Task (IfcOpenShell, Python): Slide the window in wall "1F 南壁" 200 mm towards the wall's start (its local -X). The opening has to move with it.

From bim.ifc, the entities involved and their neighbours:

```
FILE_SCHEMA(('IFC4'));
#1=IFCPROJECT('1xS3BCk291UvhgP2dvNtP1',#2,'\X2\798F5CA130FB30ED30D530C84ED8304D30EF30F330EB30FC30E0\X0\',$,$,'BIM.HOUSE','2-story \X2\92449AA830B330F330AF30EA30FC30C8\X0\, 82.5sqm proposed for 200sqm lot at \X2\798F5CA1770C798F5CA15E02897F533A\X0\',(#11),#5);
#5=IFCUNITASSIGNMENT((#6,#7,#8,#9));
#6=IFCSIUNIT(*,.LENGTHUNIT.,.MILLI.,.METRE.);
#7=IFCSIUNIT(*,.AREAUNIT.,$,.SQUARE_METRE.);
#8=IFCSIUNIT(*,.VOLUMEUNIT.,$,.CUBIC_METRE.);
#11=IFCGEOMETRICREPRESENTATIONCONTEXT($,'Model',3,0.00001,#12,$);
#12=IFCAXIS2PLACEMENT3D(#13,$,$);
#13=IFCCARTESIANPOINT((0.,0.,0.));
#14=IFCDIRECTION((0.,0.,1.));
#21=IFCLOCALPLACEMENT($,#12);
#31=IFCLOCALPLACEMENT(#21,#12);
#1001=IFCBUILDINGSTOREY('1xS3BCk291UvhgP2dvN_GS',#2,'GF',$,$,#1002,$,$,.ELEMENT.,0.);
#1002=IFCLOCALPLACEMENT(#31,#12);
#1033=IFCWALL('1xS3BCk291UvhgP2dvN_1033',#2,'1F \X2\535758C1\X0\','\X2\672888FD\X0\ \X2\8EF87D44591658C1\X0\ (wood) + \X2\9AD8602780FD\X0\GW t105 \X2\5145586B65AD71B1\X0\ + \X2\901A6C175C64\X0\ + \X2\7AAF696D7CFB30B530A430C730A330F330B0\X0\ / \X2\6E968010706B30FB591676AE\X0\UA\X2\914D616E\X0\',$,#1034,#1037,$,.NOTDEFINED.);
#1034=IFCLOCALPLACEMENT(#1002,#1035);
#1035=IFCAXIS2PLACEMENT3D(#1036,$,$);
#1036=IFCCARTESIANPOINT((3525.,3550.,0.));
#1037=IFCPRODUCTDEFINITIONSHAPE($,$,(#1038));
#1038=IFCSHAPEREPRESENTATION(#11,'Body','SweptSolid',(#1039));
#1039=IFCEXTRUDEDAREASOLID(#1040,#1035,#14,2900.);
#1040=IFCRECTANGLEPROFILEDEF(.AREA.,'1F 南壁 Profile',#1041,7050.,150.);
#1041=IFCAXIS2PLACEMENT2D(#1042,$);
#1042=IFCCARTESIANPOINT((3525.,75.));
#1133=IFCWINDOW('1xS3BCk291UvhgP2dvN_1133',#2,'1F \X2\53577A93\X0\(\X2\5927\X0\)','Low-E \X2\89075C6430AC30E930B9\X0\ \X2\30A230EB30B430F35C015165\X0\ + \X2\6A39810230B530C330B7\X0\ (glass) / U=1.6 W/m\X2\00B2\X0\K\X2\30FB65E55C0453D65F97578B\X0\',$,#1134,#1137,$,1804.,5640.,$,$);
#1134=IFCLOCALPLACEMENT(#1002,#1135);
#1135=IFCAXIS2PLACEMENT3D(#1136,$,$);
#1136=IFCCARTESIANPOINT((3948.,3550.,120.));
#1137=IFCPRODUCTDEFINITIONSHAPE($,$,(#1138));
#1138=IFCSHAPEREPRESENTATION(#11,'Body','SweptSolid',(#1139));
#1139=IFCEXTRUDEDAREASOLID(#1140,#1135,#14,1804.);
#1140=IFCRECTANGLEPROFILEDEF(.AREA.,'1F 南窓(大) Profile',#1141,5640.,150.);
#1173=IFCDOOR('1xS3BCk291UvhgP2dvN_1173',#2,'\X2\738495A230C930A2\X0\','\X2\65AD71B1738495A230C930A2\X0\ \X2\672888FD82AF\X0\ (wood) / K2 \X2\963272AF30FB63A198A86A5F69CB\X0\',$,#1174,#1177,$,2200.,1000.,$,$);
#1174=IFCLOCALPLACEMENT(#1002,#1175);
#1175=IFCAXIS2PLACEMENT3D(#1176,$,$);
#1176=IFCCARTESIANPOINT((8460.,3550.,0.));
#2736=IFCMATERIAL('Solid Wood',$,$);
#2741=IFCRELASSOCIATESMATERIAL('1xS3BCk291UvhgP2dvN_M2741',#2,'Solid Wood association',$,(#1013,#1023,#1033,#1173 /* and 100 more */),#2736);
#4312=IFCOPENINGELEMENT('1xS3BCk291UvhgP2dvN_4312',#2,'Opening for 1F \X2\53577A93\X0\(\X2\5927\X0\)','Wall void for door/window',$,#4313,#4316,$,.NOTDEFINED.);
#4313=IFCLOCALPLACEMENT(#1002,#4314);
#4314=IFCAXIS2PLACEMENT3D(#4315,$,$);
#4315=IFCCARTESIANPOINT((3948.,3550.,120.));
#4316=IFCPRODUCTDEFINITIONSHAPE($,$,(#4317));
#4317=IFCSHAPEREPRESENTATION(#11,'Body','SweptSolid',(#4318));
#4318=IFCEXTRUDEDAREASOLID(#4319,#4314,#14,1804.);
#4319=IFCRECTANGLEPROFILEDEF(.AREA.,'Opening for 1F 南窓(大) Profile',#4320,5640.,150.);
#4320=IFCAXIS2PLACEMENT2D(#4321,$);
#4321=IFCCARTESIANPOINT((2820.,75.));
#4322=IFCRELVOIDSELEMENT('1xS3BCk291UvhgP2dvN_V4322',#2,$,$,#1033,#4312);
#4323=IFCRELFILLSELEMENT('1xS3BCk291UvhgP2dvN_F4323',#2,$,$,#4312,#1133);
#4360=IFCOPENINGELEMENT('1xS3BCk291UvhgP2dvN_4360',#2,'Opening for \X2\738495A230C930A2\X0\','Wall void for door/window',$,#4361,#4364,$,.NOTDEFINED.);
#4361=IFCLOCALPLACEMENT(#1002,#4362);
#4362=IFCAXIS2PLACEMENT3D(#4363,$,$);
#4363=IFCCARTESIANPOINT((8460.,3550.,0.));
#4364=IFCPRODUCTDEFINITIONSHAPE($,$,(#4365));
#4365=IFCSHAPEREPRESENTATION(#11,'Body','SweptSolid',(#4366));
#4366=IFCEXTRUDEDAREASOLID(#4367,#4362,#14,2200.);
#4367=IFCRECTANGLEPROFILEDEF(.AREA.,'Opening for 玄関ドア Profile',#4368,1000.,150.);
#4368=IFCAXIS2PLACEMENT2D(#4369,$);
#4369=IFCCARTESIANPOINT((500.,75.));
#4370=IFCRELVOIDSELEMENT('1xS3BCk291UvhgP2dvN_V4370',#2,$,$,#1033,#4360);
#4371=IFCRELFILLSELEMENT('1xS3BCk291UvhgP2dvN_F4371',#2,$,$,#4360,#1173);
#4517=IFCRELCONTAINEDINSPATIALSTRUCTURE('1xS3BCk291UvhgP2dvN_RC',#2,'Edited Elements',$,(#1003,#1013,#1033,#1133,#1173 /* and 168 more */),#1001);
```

```python
import ifcopenshell
import ifcopenshell.api.geometry
import ifcopenshell.util.placement

model = ifcopenshell.open("bim.ifc")

window = model.by_guid("1xS3BCk291UvhgP2dvN_1133")
opening = window.FillsVoids[0].RelatingOpeningElement
wall = opening.VoidsElements[0].RelatingBuildingElement

wall_matrix = ifcopenshell.util.placement.get_local_placement(wall.ObjectPlacement)
shift = wall_matrix[:3, 0] * -200.0
before = ifcopenshell.util.placement.get_local_placement(window.ObjectPlacement)[:3, 3].copy()

# The window is not placed relative to its opening, so move both.
for product in (opening, window):
    matrix = ifcopenshell.util.placement.get_local_placement(product.ObjectPlacement)
    matrix[:3, 3] += shift
    ifcopenshell.api.geometry.edit_object_placement(model, product=product, matrix=matrix, is_si=False)

after = ifcopenshell.util.placement.get_local_placement(window.ObjectPlacement)[:3, 3]
print("window moved by", (after - before).round(3) + 0.0)

model.write("bim_v2.ifc")
```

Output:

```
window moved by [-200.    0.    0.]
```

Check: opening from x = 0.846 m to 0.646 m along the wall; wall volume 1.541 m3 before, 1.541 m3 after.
